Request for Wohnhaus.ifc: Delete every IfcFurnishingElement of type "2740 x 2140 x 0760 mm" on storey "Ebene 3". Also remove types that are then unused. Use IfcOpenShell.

First a look at what the model holds.

```python
import ifcopenshell
import ifcopenshell.util.element

model = ifcopenshell.open("Wohnhaus.ifc")
print(model.schema)
storey = next(s for s in model.by_type("IfcBuildingStorey") if s.Name == "Ebene 3")
furniture = [e for e in ifcopenshell.util.element.get_decomposition(storey) if e.is_a("IfcFurnishingElement")]
seen = {}
for e in furniture:
    element_type = ifcopenshell.util.element.get_type(e)
    name = element_type.Name if element_type not in (None, e) else None
    seen[name] = seen.get(name, 0) + 1
for name, count in sorted(seen.items(), key=str):
    print(count, "x", name)
```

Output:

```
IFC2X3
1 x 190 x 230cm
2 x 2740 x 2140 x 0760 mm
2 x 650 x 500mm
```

```python
import ifcopenshell
import ifcopenshell.api.root
import ifcopenshell.util.element

model = ifcopenshell.open("Wohnhaus.ifc")

storey = next(s for s in model.by_type("IfcBuildingStorey") if s.Name == "Ebene 3")
furniture = [e for e in ifcopenshell.util.element.get_decomposition(storey) if e.is_a("IfcFurnishingElement")]
targets = [e for e in furniture if (t := ifcopenshell.util.element.get_type(e)) not in (None, e) and t.Name == "2740 x 2140 x 0760 mm"]
types = {ifcopenshell.util.element.get_type(e) for e in targets} - {None, *targets}

for e in targets:
    ifcopenshell.api.root.remove_product(model, product=e)
print(len(targets), "removed")

unused = [t for t in types if not ifcopenshell.util.element.get_types(t)]
for t in unused:
    ifcopenshell.api.root.remove_product(model, product=t)
print(len(unused), "unused types removed")

model.write("Wohnhaus_edited.ifc")
```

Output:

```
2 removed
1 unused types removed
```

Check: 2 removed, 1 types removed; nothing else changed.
